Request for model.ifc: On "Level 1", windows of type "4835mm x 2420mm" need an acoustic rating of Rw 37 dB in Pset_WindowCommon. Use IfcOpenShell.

First a look at what the model holds.

```python
import ifcopenshell
import ifcopenshell.util.element

model = ifcopenshell.open("model.ifc")
print(model.schema)
storey = next(s for s in model.by_type("IfcBuildingStorey") if s.Name == "Level 1")
windows = [e for e in ifcopenshell.util.element.get_decomposition(storey) if e.is_a("IfcWindow")]
seen = {}
for e in windows:
    element_type = ifcopenshell.util.element.get_type(e)
    key = (element_type.Name if element_type != e and element_type else None, ifcopenshell.util.element.get_pset(e, "Pset_WindowCommon", "AcousticRating"))
    seen[key] = seen.get(key, 0) + 1
for (name, value), count in sorted(seen.items(), key=str):
    print(count, "x", name, "|", value)
```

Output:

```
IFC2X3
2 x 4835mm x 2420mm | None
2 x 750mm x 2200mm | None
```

```python
import ifcopenshell
import ifcopenshell.api.pset
import ifcopenshell.util.element

model = ifcopenshell.open("model.ifc")

storey = next(s for s in model.by_type("IfcBuildingStorey") if s.Name == "Level 1")
windows = [e for e in ifcopenshell.util.element.get_decomposition(storey) if e.is_a("IfcWindow")]

count = 0
for e in windows:
    element_type = ifcopenshell.util.element.get_type(e)
    if element_type in (None, e) or element_type.Name != "4835mm x 2420mm":
        continue
    # add_pset returns the element's existing set when there is one.
    pset = ifcopenshell.api.pset.add_pset(model, product=e, name="Pset_WindowCommon")
    ifcopenshell.api.pset.edit_pset(model, pset=pset, properties={"AcousticRating": "Rw 37 dB"})
    count += 1

print(count, "windows updated")

model.write("model_rev.ifc")
```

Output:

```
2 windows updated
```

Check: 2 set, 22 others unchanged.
